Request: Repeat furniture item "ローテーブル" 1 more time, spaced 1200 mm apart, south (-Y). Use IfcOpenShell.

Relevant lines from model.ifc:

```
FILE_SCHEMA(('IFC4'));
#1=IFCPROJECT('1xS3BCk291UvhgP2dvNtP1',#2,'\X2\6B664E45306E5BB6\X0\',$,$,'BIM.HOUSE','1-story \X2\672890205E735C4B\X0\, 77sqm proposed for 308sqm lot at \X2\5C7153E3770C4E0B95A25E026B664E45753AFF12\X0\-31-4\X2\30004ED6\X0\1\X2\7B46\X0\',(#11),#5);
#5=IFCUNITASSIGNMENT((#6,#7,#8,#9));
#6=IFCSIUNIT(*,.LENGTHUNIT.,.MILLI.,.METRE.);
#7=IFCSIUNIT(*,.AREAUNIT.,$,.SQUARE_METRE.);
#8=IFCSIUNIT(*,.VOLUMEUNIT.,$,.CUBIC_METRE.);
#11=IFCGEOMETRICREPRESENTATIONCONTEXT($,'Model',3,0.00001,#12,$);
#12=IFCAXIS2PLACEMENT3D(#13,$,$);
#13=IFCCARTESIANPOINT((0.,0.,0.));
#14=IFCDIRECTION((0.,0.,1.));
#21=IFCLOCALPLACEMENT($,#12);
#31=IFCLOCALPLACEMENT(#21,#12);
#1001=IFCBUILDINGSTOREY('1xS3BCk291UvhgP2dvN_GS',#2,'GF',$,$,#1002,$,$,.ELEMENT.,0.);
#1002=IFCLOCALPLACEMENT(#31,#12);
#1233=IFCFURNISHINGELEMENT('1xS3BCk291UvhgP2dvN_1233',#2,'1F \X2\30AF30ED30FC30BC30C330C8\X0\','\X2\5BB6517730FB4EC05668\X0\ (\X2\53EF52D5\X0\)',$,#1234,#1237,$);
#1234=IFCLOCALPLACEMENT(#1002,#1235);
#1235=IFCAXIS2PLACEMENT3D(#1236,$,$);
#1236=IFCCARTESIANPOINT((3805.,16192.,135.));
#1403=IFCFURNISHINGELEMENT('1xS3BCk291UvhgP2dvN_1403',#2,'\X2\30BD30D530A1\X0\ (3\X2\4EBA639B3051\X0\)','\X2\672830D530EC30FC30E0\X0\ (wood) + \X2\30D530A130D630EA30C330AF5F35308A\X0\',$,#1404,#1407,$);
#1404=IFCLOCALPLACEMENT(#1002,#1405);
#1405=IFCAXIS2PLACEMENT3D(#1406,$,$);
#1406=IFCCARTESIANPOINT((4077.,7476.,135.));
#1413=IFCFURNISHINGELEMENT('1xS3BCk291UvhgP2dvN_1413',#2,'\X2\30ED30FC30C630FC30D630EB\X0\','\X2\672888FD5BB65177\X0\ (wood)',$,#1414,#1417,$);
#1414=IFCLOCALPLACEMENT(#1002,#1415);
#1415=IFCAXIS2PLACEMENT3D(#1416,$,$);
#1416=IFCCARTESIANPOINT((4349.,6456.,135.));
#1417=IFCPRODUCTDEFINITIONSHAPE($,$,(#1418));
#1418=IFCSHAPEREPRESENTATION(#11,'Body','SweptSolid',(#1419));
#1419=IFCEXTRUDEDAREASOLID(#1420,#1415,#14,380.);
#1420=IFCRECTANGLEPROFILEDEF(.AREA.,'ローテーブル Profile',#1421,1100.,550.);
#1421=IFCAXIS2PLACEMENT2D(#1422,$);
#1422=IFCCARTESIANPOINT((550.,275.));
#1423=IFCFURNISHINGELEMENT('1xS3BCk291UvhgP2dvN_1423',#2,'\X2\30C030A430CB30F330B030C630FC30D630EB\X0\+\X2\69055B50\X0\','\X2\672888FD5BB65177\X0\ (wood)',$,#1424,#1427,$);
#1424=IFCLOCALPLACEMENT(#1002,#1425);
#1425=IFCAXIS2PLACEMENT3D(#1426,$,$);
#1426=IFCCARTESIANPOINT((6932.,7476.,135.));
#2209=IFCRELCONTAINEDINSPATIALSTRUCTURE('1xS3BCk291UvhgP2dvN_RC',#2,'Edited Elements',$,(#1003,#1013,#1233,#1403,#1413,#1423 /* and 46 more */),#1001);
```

```python
import numpy as np
import ifcopenshell
import ifcopenshell.api.geometry
import ifcopenshell.api.root
import ifcopenshell.util.element
import ifcopenshell.util.placement

model = ifcopenshell.open("model.ifc")


def reuse_history(source, copy):
    """copy_class also copies each property set's owner history, people and application; keep the originals."""
    for rel in copy.IsDefinedBy:
        if rel.is_a("IfcRelDefinesByProperties") and (history := rel.RelatingPropertyDefinition.OwnerHistory):
            rel.RelatingPropertyDefinition.OwnerHistory = source.OwnerHistory
            ifcopenshell.util.element.remove_deep2(model, history)


source = model.by_guid("1xS3BCk291UvhgP2dvN_1413")
base = ifcopenshell.util.placement.get_local_placement(source.ObjectPlacement)
step = np.array([0.0, -1.0, 0.0]) * 1200.0

for i in range(1, 2):
    copy = ifcopenshell.api.root.copy_class(model, product=source)
    copy.Representation = ifcopenshell.util.element.copy_deep(
        model, source.Representation, exclude=["IfcGeometricRepresentationContext", "IfcRepresentationMap"]
    )
    reuse_history(source, copy)
    matrix = base.copy()
    matrix[:3, 3] += i * step
    print("added at", matrix[:3, 3].round(3) + 0.0)
    ifcopenshell.api.geometry.edit_object_placement(model, product=copy, matrix=matrix, is_si=False)

model.write("model-out.ifc")
```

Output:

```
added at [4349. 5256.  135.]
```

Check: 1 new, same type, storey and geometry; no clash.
